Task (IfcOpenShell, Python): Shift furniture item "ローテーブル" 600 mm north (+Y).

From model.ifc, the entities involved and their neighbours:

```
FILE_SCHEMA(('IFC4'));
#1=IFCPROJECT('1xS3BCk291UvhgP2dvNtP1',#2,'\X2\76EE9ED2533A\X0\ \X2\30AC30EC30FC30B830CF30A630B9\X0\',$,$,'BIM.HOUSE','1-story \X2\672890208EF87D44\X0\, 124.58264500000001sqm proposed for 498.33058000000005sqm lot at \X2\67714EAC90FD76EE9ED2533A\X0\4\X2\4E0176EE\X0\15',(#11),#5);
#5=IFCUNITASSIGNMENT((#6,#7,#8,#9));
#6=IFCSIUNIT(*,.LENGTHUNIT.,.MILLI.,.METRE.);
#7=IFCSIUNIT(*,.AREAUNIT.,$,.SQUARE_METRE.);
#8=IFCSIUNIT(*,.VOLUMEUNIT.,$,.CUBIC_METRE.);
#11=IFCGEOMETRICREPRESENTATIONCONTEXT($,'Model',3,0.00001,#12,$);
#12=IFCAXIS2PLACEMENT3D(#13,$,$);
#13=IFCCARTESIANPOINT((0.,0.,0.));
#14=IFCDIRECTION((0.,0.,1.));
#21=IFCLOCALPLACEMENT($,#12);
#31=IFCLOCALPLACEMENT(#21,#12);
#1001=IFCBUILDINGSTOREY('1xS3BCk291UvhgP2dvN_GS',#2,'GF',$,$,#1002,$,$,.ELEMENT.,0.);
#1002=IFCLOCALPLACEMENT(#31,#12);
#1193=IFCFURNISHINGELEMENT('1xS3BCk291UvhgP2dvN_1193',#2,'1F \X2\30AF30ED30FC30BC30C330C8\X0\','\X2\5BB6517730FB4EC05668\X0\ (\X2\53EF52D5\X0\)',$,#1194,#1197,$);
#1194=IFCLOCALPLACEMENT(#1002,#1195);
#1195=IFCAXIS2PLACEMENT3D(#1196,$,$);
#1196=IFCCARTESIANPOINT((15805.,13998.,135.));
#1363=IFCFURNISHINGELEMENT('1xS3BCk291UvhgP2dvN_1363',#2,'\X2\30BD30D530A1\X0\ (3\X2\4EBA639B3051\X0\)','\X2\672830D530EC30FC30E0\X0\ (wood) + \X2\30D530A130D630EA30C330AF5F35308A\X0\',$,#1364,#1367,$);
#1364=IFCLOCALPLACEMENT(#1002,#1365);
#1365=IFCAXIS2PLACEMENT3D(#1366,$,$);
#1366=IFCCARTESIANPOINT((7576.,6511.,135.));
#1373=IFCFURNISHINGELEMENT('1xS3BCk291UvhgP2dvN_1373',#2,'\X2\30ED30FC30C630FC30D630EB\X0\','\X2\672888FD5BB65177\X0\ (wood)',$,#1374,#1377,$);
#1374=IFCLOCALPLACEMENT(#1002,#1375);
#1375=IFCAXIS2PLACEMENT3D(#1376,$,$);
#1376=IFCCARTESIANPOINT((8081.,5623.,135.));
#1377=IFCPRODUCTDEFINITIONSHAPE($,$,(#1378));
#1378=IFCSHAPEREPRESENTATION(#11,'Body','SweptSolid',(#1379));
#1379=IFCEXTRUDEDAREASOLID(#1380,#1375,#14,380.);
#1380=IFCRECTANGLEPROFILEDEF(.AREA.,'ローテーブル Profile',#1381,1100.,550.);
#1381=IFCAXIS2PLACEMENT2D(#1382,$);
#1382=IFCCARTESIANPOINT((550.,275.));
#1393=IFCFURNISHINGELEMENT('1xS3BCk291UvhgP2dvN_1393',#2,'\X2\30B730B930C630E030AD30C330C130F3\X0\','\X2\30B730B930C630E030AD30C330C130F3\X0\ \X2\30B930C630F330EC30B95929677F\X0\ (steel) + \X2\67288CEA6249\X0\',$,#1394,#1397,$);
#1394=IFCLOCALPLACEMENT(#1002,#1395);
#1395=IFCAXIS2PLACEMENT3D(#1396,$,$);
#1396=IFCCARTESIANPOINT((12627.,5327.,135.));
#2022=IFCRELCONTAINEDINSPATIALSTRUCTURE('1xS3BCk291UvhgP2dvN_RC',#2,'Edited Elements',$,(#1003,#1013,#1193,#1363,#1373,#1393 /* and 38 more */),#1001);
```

```python
import ifcopenshell
import ifcopenshell.api.geometry
import ifcopenshell.util.placement
import ifcopenshell.util.unit

model = ifcopenshell.open("model.ifc")
unit_scale = ifcopenshell.util.unit.calculate_unit_scale(model)

item = model.by_guid("1xS3BCk291UvhgP2dvN_1373")
matrix = ifcopenshell.util.placement.get_local_placement(item.ObjectPlacement)
matrix[1, 3] += 0.6 / unit_scale
ifcopenshell.api.geometry.edit_object_placement(model, product=item, matrix=matrix, is_si=False)

print(ifcopenshell.util.placement.get_local_placement(item.ObjectPlacement).round(3) + 0.0)

model.write("model_updated.ifc")
```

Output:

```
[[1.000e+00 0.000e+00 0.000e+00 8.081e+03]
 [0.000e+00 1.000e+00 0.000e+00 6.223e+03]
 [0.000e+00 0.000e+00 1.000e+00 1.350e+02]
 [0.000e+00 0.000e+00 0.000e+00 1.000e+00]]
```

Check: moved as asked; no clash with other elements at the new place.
